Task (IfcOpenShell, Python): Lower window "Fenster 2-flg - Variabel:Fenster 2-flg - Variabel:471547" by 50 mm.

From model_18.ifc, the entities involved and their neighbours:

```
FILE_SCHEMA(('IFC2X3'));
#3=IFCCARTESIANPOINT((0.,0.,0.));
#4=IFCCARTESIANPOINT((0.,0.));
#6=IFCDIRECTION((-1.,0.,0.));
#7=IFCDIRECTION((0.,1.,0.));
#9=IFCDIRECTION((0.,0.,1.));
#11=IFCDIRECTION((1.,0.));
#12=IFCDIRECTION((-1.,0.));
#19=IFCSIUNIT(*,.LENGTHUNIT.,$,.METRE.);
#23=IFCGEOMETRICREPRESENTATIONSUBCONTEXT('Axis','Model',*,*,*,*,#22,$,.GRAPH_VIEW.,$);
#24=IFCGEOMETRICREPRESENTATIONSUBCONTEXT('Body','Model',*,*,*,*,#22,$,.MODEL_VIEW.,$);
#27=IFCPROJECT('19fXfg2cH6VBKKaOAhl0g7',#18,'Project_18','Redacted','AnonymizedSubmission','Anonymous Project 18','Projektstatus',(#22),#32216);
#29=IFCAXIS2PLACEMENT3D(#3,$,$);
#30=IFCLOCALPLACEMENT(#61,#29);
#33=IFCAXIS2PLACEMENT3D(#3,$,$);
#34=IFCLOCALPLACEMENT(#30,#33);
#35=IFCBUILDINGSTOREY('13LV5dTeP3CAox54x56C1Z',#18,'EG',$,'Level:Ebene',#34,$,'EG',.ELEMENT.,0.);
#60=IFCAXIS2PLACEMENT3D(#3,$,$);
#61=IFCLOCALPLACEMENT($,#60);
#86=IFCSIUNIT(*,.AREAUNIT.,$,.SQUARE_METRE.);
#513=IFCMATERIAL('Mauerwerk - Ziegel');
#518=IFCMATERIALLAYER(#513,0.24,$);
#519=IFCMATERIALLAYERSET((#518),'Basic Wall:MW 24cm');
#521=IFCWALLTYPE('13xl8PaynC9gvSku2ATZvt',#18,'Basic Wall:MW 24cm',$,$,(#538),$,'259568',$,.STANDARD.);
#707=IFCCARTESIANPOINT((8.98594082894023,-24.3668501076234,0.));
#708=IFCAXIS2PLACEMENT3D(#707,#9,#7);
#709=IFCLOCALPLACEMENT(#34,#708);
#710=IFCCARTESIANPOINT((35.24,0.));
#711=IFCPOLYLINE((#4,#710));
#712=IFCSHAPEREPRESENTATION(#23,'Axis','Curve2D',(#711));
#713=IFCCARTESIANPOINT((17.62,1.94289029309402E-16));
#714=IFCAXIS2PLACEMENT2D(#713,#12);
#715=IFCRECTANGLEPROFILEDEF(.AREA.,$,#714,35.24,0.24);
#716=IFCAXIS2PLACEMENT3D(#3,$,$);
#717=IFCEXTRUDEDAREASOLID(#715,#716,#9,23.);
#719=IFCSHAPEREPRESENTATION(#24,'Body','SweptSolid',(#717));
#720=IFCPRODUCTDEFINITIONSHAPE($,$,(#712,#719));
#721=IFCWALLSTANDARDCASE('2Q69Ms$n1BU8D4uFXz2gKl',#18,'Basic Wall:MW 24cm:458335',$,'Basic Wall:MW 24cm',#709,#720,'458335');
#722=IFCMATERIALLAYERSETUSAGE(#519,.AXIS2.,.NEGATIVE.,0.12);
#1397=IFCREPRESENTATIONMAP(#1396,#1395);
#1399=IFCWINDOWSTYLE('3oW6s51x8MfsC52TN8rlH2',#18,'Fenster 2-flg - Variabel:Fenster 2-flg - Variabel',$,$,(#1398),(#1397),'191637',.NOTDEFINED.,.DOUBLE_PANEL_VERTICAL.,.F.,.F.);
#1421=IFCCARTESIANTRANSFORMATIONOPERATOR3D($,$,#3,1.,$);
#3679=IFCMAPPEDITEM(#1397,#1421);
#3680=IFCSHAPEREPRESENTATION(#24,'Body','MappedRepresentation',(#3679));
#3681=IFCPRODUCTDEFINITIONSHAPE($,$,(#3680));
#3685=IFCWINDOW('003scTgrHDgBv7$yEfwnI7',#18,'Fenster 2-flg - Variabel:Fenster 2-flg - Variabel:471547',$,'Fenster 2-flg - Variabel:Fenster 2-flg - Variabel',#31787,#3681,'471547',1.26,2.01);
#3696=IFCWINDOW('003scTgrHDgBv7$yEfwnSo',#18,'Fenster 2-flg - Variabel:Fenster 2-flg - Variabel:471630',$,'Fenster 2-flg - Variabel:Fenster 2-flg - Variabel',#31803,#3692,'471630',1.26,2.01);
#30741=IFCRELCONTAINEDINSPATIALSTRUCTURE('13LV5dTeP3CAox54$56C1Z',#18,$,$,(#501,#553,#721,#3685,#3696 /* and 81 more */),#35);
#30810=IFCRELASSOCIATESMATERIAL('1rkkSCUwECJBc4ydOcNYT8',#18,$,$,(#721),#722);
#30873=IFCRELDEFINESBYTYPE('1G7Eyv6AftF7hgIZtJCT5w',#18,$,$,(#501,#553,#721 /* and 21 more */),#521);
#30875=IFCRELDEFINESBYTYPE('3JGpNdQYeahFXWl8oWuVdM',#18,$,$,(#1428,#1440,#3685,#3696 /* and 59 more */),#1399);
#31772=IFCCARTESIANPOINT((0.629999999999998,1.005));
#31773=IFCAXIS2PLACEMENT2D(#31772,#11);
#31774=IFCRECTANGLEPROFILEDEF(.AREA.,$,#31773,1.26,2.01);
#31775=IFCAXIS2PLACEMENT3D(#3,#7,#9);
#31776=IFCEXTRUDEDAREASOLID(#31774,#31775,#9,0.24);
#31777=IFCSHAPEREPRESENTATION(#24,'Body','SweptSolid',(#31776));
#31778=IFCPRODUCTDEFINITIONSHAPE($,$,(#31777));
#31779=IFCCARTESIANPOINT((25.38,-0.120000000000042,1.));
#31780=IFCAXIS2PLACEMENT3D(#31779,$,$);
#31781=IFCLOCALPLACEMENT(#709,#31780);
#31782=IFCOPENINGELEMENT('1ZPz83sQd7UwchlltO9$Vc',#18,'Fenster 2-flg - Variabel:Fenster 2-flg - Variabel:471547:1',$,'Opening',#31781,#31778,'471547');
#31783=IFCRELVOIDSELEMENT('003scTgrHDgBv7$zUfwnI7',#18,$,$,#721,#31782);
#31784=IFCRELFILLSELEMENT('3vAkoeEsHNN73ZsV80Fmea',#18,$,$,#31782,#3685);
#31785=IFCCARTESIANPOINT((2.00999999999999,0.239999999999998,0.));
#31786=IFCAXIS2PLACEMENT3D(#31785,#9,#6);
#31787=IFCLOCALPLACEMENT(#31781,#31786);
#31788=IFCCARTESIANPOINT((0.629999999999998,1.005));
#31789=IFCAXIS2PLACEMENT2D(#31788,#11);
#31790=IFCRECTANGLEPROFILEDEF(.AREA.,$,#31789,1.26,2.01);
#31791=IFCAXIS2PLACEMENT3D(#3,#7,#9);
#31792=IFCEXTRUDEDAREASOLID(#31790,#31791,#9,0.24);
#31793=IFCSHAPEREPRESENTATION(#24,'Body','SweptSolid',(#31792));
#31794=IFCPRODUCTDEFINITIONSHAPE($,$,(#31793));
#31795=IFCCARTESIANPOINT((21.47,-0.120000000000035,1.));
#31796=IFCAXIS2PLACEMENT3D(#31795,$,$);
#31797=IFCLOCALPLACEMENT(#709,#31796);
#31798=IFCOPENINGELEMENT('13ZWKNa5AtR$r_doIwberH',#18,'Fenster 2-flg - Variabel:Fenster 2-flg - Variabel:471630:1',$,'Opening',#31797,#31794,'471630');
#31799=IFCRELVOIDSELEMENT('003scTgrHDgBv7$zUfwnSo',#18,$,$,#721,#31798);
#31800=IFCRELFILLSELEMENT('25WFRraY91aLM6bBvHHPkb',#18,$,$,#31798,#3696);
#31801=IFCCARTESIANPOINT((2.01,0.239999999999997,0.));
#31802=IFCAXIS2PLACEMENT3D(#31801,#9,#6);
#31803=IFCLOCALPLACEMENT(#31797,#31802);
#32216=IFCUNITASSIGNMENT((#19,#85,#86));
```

```python
import numpy as np
import ifcopenshell
import ifcopenshell.api.geometry
import ifcopenshell.util.placement
import ifcopenshell.util.unit

model = ifcopenshell.open("model_18.ifc")
unit_scale = ifcopenshell.util.unit.calculate_unit_scale(model)

window = model.by_guid("003scTgrHDgBv7$yEfwnI7")
opening = window.FillsVoids[0].RelatingOpeningElement
dz = -0.05

shift = np.array([0.0, 0.0, dz])
# The window is placed relative to its opening, so it follows when the opening moves.
matrix = ifcopenshell.util.placement.get_local_placement(opening.ObjectPlacement)
matrix[:3, 3] += shift
ifcopenshell.api.geometry.edit_object_placement(
    model, product=opening, matrix=matrix, is_si=False, should_transform_children=True
)

print(f"moved by {dz * unit_scale:+.3f} m")

model.write("model_18_rev.ifc")
```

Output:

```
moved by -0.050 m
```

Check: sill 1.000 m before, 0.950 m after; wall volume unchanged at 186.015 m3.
